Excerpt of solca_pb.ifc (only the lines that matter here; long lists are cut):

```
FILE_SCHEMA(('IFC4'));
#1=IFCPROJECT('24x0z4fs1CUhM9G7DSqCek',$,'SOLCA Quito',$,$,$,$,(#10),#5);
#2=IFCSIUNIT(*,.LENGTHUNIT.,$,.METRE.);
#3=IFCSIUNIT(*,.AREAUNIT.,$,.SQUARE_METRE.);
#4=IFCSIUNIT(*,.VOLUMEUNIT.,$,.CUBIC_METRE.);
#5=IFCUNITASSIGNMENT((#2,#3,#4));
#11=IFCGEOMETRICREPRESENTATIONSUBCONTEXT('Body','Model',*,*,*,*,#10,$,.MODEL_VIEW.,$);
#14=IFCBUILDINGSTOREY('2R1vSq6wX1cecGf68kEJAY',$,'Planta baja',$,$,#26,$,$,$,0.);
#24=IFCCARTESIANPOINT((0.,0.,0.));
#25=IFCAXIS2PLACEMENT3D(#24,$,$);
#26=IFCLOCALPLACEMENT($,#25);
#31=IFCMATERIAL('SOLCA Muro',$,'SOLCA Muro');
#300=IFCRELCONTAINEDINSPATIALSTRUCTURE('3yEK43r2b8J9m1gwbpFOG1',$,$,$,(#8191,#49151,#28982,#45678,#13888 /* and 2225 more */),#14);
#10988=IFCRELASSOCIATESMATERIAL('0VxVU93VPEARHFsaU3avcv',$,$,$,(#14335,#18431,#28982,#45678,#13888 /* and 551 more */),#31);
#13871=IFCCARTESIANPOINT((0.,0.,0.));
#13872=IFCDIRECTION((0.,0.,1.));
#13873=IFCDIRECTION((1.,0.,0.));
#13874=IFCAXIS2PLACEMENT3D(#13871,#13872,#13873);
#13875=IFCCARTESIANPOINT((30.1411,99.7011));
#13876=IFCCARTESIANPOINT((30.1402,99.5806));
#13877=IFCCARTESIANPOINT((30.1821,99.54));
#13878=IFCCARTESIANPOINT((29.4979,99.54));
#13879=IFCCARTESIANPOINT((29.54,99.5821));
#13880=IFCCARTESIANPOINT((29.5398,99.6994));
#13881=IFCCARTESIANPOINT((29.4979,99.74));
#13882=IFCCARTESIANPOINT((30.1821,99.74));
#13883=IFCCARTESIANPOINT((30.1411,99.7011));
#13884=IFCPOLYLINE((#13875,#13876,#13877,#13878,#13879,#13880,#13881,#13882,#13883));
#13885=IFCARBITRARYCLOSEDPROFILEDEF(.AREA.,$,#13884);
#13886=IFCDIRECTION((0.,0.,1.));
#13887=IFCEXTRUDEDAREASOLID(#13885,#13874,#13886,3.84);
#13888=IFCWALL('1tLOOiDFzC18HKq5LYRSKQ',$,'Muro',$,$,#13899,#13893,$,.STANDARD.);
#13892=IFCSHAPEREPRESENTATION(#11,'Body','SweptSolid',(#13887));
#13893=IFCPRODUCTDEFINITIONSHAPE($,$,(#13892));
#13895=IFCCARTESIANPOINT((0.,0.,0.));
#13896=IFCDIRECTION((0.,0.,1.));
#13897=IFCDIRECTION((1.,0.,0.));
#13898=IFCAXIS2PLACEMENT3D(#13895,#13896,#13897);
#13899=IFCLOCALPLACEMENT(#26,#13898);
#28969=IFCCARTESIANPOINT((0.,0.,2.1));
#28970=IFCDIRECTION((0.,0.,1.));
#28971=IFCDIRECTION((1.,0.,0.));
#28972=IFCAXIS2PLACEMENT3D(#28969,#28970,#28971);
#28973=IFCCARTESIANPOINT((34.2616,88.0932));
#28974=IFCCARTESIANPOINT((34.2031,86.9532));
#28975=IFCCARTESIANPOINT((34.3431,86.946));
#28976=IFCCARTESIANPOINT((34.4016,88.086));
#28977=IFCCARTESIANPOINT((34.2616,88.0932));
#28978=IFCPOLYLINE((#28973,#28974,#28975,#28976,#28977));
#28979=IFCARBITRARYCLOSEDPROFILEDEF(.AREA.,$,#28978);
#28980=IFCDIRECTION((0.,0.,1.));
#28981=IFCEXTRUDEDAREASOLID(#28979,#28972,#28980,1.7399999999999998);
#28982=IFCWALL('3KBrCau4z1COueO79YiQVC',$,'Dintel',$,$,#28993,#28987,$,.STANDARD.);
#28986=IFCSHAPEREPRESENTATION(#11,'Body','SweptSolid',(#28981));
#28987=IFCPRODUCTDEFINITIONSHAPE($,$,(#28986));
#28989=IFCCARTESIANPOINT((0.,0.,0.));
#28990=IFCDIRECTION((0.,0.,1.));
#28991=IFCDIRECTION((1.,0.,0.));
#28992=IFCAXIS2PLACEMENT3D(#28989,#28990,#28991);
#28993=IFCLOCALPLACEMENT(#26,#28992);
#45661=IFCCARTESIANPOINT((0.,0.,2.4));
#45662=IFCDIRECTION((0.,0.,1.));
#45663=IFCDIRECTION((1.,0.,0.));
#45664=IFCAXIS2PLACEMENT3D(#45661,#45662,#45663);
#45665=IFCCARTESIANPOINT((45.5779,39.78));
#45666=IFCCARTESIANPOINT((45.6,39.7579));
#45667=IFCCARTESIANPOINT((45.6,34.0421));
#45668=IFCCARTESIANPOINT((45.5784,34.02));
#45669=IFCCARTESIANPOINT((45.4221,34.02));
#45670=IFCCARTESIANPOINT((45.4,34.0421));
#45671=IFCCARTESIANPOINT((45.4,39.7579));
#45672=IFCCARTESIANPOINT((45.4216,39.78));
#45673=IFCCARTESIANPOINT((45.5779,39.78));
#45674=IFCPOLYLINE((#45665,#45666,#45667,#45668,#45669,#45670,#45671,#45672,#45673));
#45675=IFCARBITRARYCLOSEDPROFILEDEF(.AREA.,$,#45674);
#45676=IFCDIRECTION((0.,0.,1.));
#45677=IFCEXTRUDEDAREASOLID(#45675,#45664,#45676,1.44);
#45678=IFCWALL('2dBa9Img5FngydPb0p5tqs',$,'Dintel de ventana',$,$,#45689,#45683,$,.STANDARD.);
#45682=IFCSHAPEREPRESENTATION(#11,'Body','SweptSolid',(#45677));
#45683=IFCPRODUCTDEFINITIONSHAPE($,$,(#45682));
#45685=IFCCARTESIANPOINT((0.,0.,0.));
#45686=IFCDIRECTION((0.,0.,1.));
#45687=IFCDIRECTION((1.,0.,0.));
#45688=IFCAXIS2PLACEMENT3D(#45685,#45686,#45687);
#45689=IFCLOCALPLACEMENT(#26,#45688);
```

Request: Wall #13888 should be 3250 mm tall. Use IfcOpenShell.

```python
import ifcopenshell
import ifcopenshell.geom
import ifcopenshell.util.representation
import ifcopenshell.util.shape
import ifcopenshell.util.unit

model = ifcopenshell.open("solca_pb.ifc")
unit_scale = ifcopenshell.util.unit.calculate_unit_scale(model)
settings = ifcopenshell.geom.settings()


def volume(element):
    """Net volume in cubic metres, openings subtracted."""
    shape = ifcopenshell.geom.create_shape(settings, element)
    return ifcopenshell.util.shape.get_volume(shape.geometry)


wall = model.by_guid("1tLOOiDFzC18HKq5LYRSKQ")
before = volume(wall)

body = ifcopenshell.util.representation.get_representation(wall, "Model", "Body")
solid = body.Items[0]
old_height = solid.Depth
solid.Depth = 3.25 / unit_scale
after = volume(wall)

print(f"height {old_height:g} -> {solid.Depth:g}, volume {before:.3f} -> {after:.3f} m3")

model.write("solca_pb_rev.ifc")
```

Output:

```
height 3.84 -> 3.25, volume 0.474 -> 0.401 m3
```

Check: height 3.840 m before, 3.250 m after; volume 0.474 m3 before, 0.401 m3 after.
